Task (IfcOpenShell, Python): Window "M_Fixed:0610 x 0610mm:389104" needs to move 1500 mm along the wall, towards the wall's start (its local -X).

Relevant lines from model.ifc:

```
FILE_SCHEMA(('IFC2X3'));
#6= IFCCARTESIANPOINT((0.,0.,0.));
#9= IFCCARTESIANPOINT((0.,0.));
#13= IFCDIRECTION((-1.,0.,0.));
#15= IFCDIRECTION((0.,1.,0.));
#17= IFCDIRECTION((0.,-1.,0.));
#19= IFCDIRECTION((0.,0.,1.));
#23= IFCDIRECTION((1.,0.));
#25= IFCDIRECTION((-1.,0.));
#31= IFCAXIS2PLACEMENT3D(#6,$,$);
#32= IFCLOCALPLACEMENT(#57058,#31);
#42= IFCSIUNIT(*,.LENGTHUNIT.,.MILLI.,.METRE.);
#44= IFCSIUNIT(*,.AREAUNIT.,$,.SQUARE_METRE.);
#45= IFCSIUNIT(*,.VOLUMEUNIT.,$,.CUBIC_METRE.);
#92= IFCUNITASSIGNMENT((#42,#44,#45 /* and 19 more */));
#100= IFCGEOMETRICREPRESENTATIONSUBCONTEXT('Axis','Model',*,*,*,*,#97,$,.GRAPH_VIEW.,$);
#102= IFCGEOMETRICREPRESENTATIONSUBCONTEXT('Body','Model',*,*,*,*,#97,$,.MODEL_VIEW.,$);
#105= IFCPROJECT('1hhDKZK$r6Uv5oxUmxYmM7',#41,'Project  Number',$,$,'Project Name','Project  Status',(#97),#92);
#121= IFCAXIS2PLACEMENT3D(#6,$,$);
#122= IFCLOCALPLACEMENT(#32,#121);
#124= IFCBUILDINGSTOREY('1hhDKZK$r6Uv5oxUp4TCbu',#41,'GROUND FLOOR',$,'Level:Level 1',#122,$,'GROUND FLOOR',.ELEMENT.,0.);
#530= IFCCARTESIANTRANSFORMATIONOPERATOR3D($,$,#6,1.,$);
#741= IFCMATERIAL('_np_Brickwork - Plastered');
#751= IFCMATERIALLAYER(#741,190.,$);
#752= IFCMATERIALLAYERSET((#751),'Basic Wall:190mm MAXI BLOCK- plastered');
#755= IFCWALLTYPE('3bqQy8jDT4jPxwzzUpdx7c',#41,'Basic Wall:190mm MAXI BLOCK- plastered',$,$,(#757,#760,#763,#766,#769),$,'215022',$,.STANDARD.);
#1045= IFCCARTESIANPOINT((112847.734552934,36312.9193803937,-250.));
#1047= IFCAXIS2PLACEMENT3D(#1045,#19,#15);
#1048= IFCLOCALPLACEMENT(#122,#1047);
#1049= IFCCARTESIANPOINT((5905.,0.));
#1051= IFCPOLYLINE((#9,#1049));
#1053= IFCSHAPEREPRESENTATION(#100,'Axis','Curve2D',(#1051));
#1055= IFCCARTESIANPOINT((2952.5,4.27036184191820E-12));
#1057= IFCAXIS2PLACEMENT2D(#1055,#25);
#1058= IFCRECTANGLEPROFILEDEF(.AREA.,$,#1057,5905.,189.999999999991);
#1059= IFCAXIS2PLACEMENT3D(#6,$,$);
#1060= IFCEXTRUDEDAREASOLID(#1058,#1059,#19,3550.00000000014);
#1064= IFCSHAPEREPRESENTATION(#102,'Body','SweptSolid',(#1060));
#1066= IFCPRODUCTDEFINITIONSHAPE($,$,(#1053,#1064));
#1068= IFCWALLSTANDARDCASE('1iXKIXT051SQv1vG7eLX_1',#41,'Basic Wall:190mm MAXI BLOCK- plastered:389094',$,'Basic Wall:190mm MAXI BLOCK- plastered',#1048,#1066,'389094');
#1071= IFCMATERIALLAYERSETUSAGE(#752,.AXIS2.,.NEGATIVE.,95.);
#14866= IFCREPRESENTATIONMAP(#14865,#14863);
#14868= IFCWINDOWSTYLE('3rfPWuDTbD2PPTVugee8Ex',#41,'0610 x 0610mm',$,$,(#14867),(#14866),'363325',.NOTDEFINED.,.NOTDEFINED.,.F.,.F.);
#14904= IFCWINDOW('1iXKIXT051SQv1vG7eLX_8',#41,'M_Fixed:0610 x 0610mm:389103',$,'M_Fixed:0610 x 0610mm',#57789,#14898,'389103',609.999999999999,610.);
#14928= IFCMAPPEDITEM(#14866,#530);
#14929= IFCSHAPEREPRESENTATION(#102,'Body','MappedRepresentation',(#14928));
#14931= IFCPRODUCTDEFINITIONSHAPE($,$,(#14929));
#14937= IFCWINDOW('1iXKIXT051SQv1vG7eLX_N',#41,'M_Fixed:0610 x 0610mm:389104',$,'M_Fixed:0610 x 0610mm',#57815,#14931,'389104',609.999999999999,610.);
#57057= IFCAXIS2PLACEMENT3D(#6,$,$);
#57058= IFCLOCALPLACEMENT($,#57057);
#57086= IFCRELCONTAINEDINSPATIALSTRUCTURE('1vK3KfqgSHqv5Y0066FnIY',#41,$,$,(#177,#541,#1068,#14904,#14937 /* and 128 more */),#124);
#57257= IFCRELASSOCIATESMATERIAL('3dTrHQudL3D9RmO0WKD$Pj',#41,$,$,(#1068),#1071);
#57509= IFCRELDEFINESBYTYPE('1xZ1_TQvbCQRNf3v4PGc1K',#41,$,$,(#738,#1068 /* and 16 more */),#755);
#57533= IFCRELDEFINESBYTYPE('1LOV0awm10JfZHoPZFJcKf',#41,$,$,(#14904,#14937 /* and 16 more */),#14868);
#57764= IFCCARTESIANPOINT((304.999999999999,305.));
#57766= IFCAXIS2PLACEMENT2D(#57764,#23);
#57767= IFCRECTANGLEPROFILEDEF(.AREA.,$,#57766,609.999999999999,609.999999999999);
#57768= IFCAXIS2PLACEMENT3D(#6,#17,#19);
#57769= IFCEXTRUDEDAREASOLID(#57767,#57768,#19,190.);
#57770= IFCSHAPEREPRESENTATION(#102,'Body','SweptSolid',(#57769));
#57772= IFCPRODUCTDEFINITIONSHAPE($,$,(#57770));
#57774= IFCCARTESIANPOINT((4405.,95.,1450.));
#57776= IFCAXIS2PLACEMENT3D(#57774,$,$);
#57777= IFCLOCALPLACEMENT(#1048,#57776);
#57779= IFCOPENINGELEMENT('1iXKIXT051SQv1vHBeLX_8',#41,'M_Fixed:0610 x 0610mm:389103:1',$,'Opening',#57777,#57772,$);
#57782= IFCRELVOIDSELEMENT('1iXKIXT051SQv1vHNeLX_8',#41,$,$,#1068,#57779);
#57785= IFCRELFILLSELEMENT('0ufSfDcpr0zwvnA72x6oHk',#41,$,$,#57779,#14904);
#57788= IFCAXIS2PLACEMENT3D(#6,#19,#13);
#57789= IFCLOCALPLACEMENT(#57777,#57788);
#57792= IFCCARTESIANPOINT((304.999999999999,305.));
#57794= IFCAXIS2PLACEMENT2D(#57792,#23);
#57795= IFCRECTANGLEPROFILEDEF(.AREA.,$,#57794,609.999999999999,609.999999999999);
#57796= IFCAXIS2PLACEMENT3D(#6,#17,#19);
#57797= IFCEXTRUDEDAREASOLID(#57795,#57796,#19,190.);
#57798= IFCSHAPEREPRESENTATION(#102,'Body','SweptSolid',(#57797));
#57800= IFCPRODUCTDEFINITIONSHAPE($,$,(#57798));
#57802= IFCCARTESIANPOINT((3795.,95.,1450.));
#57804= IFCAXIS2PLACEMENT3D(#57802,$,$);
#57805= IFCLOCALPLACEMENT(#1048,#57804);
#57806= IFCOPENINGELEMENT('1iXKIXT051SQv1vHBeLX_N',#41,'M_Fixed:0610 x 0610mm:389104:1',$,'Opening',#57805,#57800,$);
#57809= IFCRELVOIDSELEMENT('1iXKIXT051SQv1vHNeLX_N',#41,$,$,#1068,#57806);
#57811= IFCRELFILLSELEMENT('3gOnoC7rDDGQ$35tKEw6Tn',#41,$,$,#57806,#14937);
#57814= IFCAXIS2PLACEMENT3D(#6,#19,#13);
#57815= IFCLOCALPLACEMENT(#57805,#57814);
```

```python
import ifcopenshell
import ifcopenshell.api.geometry
import ifcopenshell.util.placement
import ifcopenshell.util.unit

model = ifcopenshell.open("model.ifc")
unit_scale = ifcopenshell.util.unit.calculate_unit_scale(model)

window = model.by_guid("1iXKIXT051SQv1vG7eLX_N")
opening = window.FillsVoids[0].RelatingOpeningElement
wall = opening.VoidsElements[0].RelatingBuildingElement

wall_matrix = ifcopenshell.util.placement.get_local_placement(wall.ObjectPlacement)
shift = wall_matrix[:3, 0] * -1.5 / unit_scale
before = ifcopenshell.util.placement.get_local_placement(window.ObjectPlacement)[:3, 3].copy()

# The window is placed relative to its opening, so it follows when the opening moves.
matrix = ifcopenshell.util.placement.get_local_placement(opening.ObjectPlacement)
matrix[:3, 3] += shift
ifcopenshell.api.geometry.edit_object_placement(
    model, product=opening, matrix=matrix, is_si=False, should_transform_children=True
)

after = ifcopenshell.util.placement.get_local_placement(window.ObjectPlacement)[:3, 3]
print("window moved by", (after - before).round(3) + 0.0)

model.write("model_edited.ifc")
```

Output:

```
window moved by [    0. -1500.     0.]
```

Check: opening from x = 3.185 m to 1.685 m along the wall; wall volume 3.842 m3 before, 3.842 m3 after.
